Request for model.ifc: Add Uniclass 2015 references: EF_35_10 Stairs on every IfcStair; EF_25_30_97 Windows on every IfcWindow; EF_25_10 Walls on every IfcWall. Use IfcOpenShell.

First a look at what the model holds.

```python
import ifcopenshell

model = ifcopenshell.open("model.ifc")
print(model.schema)
print("classifications:", [c.Name for c in model.by_type("IfcClassification")])
for ifc_class in ("IfcDoor", "IfcRoof", "IfcStair", "IfcWall", "IfcWindow"):
    print(ifc_class, len(model.by_type(ifc_class)))
```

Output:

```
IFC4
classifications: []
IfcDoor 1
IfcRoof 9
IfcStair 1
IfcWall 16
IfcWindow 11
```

```python
import ifcopenshell
import ifcopenshell.api.classification

model = ifcopenshell.open("model.ifc")

system = ifcopenshell.api.classification.add_classification(model, classification="Uniclass 2015")

codes = {
    "IfcStair": ("EF_35_10", "Stairs"),
    "IfcWindow": ("EF_25_30_97", "Windows"),
    "IfcWall": ("EF_25_10", "Walls"),
}
for ifc_class, (code, name) in codes.items():
    products = model.by_type(ifc_class)
    ifcopenshell.api.classification.add_reference(
        model, products=products, classification=system, identification=code, name=name
    )
    print(code, len(products))

model.write("model_rev.ifc")
```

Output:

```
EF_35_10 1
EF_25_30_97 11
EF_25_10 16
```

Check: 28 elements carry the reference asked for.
